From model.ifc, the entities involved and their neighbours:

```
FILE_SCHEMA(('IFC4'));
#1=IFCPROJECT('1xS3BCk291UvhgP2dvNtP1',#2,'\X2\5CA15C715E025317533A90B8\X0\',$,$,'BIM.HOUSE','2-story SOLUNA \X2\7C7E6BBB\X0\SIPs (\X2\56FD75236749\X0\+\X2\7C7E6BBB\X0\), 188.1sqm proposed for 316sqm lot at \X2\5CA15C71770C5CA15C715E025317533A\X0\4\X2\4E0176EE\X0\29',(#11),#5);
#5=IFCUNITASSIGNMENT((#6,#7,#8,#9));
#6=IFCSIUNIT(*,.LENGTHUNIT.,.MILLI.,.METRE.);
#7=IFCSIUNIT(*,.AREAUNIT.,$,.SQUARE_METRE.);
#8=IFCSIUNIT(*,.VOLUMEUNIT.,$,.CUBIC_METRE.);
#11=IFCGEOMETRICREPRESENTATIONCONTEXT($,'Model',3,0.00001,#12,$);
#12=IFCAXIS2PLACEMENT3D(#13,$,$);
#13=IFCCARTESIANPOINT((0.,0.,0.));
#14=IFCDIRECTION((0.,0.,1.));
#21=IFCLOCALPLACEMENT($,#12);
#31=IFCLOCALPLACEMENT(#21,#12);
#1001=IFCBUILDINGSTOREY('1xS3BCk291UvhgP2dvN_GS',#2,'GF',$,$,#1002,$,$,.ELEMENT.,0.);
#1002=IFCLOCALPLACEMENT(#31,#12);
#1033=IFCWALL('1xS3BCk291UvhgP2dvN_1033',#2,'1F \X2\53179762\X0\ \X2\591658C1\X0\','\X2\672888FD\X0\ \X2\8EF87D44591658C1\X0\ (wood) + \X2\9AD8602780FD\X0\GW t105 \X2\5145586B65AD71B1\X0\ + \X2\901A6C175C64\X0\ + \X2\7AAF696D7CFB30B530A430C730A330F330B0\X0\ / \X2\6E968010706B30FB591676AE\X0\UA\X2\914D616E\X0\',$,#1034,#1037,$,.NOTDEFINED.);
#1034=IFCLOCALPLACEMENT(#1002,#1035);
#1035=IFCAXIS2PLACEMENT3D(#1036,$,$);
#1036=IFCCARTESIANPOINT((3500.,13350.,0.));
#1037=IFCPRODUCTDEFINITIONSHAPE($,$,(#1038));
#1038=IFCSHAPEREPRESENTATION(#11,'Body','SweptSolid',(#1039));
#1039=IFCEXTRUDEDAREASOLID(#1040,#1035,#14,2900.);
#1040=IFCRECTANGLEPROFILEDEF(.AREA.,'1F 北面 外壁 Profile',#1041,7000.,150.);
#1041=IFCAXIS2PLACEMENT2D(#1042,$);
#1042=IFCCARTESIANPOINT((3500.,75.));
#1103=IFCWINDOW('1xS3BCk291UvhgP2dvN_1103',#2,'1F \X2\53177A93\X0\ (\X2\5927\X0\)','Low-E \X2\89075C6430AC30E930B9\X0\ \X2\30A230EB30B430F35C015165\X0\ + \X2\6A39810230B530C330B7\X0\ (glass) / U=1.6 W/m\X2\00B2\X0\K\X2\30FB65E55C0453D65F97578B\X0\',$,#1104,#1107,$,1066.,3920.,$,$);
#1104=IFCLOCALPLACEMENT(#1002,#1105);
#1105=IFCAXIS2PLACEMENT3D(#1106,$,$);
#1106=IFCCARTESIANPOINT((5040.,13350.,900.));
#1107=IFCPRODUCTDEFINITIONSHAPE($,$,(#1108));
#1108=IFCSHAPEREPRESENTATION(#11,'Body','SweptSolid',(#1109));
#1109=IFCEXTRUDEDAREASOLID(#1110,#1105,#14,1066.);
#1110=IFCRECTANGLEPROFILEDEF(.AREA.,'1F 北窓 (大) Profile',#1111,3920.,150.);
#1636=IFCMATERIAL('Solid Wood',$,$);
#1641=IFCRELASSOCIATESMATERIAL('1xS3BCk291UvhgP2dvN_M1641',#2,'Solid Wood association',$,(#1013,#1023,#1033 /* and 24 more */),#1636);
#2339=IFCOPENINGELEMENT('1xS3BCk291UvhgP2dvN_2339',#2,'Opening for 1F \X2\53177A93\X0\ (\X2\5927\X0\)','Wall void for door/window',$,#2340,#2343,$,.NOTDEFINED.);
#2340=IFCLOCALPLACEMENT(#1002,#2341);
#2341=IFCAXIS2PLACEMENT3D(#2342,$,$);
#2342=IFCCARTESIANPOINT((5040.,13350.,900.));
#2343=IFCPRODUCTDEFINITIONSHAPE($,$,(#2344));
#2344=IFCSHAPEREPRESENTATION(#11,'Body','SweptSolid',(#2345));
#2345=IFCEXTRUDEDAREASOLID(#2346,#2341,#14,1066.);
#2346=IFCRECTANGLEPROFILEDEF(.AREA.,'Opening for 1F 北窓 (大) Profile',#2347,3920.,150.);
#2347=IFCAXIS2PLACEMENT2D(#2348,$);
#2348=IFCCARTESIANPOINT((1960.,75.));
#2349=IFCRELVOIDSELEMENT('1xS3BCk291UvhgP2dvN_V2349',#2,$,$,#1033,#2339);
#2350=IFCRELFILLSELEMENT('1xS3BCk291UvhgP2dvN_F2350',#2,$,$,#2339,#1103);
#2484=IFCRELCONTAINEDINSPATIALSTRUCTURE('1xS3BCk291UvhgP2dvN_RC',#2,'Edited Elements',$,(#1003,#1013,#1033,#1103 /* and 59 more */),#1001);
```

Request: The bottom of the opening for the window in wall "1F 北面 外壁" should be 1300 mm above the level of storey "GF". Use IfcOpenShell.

```python
import numpy as np
import ifcopenshell
import ifcopenshell.api.geometry
import ifcopenshell.geom
import ifcopenshell.util.element
import ifcopenshell.util.placement
import ifcopenshell.util.shape
import ifcopenshell.util.unit

model = ifcopenshell.open("model.ifc")
unit_scale = ifcopenshell.util.unit.calculate_unit_scale(model)

window = model.by_id(1103)
opening = window.FillsVoids[0].RelatingOpeningElement
storey = ifcopenshell.util.element.get_container(window, ifc_class="IfcBuildingStorey")
level = ifcopenshell.util.placement.get_local_placement(storey.ObjectPlacement)[2, 3]

# The opening's origin need not be at the sill, so measure its lowest point.
shape = ifcopenshell.geom.create_shape(ifcopenshell.geom.settings(), opening)
bottom = ifcopenshell.util.shape.get_shape_bottom_elevation(shape, shape.geometry) / unit_scale
dz = level + 1300.0 - bottom

shift = np.array([0.0, 0.0, dz])
# The window is not placed relative to its opening, so move both.
for product in (opening, window):
    matrix = ifcopenshell.util.placement.get_local_placement(product.ObjectPlacement)
    matrix[:3, 3] += shift
    ifcopenshell.api.geometry.edit_object_placement(model, product=product, matrix=matrix, is_si=False)

print(f"moved by {dz * unit_scale:+.3f} m")

model.write("model_rev.ifc")
```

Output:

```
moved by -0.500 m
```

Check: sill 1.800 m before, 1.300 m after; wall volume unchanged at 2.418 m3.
